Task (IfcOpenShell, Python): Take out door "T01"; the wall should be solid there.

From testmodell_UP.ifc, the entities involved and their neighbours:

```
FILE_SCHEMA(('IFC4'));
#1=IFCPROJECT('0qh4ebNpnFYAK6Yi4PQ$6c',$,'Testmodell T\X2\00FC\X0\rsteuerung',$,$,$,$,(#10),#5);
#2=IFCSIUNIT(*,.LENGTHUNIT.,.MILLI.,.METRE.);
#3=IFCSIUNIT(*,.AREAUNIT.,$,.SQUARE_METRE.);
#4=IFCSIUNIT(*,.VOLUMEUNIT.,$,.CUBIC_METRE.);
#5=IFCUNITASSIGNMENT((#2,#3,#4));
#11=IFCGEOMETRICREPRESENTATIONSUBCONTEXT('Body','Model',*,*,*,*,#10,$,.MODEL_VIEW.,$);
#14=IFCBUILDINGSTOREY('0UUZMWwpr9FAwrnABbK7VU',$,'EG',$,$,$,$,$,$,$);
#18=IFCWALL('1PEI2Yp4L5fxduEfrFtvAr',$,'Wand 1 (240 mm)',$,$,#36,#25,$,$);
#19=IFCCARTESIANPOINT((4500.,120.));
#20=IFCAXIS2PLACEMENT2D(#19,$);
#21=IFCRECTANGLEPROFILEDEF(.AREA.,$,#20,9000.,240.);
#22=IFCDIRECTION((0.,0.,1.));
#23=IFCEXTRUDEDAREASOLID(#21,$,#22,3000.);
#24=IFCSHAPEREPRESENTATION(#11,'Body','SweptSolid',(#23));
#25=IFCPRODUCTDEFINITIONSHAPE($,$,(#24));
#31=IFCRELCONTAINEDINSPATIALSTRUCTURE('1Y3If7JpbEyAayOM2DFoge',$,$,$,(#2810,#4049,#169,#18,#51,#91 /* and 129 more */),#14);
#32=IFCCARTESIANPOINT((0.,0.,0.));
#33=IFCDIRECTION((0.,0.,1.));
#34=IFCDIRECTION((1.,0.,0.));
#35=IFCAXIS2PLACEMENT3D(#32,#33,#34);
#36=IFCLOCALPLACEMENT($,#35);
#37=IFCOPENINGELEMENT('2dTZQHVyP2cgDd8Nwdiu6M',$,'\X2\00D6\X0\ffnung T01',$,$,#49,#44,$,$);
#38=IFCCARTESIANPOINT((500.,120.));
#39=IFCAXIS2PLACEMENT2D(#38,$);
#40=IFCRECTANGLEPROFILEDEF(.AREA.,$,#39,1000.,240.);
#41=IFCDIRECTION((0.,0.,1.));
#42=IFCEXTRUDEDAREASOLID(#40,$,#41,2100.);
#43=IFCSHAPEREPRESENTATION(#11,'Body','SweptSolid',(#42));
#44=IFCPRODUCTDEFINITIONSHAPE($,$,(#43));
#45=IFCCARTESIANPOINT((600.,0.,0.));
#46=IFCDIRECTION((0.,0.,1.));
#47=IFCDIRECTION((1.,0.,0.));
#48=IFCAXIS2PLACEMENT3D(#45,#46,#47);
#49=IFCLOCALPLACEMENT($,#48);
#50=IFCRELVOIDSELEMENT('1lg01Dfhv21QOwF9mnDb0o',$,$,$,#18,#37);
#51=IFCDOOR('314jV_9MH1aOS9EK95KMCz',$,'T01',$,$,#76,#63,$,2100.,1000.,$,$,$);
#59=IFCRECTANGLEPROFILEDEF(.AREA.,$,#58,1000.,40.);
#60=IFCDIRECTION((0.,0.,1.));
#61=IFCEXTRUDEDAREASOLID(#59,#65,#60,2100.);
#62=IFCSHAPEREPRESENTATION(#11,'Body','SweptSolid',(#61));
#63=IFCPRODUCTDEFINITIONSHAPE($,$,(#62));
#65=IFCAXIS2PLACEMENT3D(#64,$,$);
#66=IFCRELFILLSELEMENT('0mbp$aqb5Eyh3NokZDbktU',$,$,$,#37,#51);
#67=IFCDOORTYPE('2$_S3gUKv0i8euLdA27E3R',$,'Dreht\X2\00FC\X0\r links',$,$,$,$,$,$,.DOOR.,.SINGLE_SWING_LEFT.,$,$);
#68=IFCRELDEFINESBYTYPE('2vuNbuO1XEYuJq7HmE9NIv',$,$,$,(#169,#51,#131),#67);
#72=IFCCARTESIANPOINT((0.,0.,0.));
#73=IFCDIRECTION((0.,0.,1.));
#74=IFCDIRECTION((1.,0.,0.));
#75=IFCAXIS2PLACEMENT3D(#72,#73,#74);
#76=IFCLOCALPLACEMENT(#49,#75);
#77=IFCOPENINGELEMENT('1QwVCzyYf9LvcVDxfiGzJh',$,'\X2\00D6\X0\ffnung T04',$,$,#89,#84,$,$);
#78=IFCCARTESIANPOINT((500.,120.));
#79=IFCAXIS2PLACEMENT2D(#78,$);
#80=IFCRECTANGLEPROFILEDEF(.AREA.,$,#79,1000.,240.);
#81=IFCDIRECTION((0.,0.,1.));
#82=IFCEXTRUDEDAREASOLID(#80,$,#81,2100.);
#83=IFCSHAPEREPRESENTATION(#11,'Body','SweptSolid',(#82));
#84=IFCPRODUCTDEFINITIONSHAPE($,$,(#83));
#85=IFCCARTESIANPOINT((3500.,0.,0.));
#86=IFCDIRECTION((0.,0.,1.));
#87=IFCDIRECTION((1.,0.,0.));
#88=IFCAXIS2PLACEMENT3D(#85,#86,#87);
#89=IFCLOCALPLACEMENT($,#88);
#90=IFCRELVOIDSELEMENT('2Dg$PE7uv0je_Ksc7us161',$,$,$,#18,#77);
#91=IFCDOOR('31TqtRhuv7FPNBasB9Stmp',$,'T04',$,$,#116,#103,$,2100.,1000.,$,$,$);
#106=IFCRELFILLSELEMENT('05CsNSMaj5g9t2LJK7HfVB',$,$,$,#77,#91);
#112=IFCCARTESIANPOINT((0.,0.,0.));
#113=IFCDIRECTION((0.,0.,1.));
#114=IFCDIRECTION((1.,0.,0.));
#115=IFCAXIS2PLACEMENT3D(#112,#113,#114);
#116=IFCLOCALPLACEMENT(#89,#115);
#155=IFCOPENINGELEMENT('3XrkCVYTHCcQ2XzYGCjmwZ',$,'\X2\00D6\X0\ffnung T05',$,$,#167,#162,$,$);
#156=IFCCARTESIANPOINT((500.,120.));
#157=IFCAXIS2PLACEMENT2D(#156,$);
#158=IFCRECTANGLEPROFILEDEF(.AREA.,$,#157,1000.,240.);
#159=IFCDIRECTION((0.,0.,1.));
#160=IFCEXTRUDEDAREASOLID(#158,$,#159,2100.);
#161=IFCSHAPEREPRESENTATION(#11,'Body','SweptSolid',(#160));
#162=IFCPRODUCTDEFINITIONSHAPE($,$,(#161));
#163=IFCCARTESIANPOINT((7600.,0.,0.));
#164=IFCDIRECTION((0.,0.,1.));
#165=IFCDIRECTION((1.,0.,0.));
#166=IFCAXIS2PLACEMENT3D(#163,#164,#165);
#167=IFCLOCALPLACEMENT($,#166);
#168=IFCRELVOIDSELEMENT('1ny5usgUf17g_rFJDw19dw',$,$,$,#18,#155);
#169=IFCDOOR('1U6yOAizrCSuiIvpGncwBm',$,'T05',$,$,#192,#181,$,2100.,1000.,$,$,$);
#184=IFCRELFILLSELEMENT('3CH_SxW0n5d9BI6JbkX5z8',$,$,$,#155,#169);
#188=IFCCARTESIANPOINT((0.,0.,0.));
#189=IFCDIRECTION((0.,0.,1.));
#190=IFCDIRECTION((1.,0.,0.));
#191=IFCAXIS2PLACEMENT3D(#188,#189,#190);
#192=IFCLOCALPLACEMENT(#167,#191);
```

```python
import ifcopenshell
import ifcopenshell.api.feature
import ifcopenshell.api.root
import ifcopenshell.geom
import ifcopenshell.util.shape

model = ifcopenshell.open("testmodell_UP.ifc")
settings = ifcopenshell.geom.settings()


def volume(element):
    """Net volume in cubic metres, openings subtracted."""
    shape = ifcopenshell.geom.create_shape(settings, element)
    return ifcopenshell.util.shape.get_volume(shape.geometry)


door = model.by_guid("314jV_9MH1aOS9EK95KMCz")
opening = door.FillsVoids[0].RelatingOpeningElement
wall = opening.VoidsElements[0].RelatingBuildingElement
before = volume(wall)

ifcopenshell.api.root.remove_product(model, product=door)
ifcopenshell.api.feature.remove_feature(model, feature=opening)

after = volume(wall)

print(f"wall volume {before:.3f} -> {after:.3f} m3")

model.write("testmodell_UP_v2.ifc")
```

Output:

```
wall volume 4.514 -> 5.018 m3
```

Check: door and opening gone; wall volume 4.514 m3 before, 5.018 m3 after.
